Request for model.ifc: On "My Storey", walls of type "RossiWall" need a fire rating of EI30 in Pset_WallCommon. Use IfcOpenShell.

First a look at what the model holds.

```python
import ifcopenshell
import ifcopenshell.util.element

model = ifcopenshell.open("model.ifc")
print(model.schema)
storey = next(s for s in model.by_type("IfcBuildingStorey") if s.Name == "My Storey")
walls = [e for e in ifcopenshell.util.element.get_decomposition(storey) if e.is_a("IfcWall")]
seen = {}
for e in walls:
    element_type = ifcopenshell.util.element.get_type(e)
    key = (element_type.Name if element_type != e and element_type else None, ifcopenshell.util.element.get_pset(e, "Pset_WallCommon", "FireRating"))
    seen[key] = seen.get(key, 0) + 1
for (name, value), count in sorted(seen.items(), key=str):
    print(count, "x", name, "|", value)
```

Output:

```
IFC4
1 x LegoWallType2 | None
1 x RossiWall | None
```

```python
import ifcopenshell
import ifcopenshell.api.pset
import ifcopenshell.util.element

model = ifcopenshell.open("model.ifc")

storey = next(s for s in model.by_type("IfcBuildingStorey") if s.Name == "My Storey")
walls = [e for e in ifcopenshell.util.element.get_decomposition(storey) if e.is_a("IfcWall")]

count = 0
for e in walls:
    element_type = ifcopenshell.util.element.get_type(e)
    if element_type in (None, e) or element_type.Name != "RossiWall":
        continue
    # add_pset returns the element's existing set when there is one.
    pset = ifcopenshell.api.pset.add_pset(model, product=e, name="Pset_WallCommon")
    ifcopenshell.api.pset.edit_pset(model, pset=pset, properties={"FireRating": "EI30"})
    count += 1

print(count, "walls updated")

model.write("model_rev.ifc")
```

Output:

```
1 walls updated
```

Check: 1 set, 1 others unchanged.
